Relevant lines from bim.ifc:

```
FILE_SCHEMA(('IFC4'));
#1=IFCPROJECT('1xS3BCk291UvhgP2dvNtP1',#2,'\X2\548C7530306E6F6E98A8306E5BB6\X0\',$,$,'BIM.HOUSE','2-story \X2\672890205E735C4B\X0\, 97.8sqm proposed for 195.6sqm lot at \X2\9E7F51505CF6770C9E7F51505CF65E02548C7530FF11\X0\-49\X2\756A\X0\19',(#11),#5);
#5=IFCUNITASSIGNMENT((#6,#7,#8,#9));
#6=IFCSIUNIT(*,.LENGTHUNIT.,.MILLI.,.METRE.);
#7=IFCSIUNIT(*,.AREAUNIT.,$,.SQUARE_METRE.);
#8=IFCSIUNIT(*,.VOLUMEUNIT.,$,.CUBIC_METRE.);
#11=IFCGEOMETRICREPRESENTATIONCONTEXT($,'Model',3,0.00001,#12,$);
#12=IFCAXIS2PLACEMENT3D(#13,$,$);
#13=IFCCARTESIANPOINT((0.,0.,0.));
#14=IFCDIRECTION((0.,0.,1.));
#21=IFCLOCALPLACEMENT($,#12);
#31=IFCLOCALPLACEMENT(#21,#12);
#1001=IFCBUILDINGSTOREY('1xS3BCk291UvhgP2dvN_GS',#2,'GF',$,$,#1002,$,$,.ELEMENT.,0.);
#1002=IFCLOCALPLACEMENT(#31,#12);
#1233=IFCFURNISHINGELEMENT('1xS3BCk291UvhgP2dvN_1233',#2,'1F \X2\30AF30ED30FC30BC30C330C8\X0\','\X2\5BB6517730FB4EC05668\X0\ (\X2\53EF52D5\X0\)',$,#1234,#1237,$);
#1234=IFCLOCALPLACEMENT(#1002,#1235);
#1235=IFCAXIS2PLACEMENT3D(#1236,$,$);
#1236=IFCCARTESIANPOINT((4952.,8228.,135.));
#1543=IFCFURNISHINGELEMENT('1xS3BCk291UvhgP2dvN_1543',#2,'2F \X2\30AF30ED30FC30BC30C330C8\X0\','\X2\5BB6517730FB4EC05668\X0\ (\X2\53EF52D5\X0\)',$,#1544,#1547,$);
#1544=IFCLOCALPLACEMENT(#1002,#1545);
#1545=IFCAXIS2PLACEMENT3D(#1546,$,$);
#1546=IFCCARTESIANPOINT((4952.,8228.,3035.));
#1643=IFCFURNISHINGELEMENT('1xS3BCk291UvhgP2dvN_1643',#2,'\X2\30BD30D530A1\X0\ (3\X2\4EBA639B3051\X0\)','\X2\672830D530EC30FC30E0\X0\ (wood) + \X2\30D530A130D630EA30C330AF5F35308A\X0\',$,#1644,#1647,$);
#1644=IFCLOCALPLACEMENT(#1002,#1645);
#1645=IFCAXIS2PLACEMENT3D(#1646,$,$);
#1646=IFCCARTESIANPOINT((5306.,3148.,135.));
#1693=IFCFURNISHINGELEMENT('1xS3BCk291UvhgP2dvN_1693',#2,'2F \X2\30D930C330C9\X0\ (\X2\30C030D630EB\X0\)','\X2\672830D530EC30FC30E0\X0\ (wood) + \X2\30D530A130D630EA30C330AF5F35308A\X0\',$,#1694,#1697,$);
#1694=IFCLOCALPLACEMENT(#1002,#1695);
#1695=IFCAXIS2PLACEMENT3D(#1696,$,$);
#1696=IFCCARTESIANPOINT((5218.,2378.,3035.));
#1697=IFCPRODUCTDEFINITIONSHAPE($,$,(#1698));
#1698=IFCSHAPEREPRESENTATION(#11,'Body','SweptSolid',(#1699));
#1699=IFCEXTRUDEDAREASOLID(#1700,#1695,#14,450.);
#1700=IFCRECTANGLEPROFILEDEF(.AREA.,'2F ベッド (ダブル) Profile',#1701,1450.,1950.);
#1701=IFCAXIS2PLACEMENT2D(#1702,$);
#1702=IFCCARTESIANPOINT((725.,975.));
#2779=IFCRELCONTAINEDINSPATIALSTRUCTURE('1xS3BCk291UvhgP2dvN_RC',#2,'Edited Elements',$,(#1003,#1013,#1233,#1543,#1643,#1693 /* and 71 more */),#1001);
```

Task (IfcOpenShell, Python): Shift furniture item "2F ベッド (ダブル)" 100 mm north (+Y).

```python
import ifcopenshell
import ifcopenshell.api.geometry
import ifcopenshell.util.placement
import ifcopenshell.util.unit

model = ifcopenshell.open("bim.ifc")
unit_scale = ifcopenshell.util.unit.calculate_unit_scale(model)

item = model.by_guid("1xS3BCk291UvhgP2dvN_1693")
matrix = ifcopenshell.util.placement.get_local_placement(item.ObjectPlacement)
matrix[1, 3] += 0.1 / unit_scale
ifcopenshell.api.geometry.edit_object_placement(model, product=item, matrix=matrix, is_si=False)

print(ifcopenshell.util.placement.get_local_placement(item.ObjectPlacement).round(3) + 0.0)

model.write("bim-out.ifc")
```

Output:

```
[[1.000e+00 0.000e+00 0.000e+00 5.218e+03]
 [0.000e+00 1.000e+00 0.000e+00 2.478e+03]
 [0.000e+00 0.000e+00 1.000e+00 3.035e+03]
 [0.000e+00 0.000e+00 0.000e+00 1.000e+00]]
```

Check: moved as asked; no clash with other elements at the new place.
